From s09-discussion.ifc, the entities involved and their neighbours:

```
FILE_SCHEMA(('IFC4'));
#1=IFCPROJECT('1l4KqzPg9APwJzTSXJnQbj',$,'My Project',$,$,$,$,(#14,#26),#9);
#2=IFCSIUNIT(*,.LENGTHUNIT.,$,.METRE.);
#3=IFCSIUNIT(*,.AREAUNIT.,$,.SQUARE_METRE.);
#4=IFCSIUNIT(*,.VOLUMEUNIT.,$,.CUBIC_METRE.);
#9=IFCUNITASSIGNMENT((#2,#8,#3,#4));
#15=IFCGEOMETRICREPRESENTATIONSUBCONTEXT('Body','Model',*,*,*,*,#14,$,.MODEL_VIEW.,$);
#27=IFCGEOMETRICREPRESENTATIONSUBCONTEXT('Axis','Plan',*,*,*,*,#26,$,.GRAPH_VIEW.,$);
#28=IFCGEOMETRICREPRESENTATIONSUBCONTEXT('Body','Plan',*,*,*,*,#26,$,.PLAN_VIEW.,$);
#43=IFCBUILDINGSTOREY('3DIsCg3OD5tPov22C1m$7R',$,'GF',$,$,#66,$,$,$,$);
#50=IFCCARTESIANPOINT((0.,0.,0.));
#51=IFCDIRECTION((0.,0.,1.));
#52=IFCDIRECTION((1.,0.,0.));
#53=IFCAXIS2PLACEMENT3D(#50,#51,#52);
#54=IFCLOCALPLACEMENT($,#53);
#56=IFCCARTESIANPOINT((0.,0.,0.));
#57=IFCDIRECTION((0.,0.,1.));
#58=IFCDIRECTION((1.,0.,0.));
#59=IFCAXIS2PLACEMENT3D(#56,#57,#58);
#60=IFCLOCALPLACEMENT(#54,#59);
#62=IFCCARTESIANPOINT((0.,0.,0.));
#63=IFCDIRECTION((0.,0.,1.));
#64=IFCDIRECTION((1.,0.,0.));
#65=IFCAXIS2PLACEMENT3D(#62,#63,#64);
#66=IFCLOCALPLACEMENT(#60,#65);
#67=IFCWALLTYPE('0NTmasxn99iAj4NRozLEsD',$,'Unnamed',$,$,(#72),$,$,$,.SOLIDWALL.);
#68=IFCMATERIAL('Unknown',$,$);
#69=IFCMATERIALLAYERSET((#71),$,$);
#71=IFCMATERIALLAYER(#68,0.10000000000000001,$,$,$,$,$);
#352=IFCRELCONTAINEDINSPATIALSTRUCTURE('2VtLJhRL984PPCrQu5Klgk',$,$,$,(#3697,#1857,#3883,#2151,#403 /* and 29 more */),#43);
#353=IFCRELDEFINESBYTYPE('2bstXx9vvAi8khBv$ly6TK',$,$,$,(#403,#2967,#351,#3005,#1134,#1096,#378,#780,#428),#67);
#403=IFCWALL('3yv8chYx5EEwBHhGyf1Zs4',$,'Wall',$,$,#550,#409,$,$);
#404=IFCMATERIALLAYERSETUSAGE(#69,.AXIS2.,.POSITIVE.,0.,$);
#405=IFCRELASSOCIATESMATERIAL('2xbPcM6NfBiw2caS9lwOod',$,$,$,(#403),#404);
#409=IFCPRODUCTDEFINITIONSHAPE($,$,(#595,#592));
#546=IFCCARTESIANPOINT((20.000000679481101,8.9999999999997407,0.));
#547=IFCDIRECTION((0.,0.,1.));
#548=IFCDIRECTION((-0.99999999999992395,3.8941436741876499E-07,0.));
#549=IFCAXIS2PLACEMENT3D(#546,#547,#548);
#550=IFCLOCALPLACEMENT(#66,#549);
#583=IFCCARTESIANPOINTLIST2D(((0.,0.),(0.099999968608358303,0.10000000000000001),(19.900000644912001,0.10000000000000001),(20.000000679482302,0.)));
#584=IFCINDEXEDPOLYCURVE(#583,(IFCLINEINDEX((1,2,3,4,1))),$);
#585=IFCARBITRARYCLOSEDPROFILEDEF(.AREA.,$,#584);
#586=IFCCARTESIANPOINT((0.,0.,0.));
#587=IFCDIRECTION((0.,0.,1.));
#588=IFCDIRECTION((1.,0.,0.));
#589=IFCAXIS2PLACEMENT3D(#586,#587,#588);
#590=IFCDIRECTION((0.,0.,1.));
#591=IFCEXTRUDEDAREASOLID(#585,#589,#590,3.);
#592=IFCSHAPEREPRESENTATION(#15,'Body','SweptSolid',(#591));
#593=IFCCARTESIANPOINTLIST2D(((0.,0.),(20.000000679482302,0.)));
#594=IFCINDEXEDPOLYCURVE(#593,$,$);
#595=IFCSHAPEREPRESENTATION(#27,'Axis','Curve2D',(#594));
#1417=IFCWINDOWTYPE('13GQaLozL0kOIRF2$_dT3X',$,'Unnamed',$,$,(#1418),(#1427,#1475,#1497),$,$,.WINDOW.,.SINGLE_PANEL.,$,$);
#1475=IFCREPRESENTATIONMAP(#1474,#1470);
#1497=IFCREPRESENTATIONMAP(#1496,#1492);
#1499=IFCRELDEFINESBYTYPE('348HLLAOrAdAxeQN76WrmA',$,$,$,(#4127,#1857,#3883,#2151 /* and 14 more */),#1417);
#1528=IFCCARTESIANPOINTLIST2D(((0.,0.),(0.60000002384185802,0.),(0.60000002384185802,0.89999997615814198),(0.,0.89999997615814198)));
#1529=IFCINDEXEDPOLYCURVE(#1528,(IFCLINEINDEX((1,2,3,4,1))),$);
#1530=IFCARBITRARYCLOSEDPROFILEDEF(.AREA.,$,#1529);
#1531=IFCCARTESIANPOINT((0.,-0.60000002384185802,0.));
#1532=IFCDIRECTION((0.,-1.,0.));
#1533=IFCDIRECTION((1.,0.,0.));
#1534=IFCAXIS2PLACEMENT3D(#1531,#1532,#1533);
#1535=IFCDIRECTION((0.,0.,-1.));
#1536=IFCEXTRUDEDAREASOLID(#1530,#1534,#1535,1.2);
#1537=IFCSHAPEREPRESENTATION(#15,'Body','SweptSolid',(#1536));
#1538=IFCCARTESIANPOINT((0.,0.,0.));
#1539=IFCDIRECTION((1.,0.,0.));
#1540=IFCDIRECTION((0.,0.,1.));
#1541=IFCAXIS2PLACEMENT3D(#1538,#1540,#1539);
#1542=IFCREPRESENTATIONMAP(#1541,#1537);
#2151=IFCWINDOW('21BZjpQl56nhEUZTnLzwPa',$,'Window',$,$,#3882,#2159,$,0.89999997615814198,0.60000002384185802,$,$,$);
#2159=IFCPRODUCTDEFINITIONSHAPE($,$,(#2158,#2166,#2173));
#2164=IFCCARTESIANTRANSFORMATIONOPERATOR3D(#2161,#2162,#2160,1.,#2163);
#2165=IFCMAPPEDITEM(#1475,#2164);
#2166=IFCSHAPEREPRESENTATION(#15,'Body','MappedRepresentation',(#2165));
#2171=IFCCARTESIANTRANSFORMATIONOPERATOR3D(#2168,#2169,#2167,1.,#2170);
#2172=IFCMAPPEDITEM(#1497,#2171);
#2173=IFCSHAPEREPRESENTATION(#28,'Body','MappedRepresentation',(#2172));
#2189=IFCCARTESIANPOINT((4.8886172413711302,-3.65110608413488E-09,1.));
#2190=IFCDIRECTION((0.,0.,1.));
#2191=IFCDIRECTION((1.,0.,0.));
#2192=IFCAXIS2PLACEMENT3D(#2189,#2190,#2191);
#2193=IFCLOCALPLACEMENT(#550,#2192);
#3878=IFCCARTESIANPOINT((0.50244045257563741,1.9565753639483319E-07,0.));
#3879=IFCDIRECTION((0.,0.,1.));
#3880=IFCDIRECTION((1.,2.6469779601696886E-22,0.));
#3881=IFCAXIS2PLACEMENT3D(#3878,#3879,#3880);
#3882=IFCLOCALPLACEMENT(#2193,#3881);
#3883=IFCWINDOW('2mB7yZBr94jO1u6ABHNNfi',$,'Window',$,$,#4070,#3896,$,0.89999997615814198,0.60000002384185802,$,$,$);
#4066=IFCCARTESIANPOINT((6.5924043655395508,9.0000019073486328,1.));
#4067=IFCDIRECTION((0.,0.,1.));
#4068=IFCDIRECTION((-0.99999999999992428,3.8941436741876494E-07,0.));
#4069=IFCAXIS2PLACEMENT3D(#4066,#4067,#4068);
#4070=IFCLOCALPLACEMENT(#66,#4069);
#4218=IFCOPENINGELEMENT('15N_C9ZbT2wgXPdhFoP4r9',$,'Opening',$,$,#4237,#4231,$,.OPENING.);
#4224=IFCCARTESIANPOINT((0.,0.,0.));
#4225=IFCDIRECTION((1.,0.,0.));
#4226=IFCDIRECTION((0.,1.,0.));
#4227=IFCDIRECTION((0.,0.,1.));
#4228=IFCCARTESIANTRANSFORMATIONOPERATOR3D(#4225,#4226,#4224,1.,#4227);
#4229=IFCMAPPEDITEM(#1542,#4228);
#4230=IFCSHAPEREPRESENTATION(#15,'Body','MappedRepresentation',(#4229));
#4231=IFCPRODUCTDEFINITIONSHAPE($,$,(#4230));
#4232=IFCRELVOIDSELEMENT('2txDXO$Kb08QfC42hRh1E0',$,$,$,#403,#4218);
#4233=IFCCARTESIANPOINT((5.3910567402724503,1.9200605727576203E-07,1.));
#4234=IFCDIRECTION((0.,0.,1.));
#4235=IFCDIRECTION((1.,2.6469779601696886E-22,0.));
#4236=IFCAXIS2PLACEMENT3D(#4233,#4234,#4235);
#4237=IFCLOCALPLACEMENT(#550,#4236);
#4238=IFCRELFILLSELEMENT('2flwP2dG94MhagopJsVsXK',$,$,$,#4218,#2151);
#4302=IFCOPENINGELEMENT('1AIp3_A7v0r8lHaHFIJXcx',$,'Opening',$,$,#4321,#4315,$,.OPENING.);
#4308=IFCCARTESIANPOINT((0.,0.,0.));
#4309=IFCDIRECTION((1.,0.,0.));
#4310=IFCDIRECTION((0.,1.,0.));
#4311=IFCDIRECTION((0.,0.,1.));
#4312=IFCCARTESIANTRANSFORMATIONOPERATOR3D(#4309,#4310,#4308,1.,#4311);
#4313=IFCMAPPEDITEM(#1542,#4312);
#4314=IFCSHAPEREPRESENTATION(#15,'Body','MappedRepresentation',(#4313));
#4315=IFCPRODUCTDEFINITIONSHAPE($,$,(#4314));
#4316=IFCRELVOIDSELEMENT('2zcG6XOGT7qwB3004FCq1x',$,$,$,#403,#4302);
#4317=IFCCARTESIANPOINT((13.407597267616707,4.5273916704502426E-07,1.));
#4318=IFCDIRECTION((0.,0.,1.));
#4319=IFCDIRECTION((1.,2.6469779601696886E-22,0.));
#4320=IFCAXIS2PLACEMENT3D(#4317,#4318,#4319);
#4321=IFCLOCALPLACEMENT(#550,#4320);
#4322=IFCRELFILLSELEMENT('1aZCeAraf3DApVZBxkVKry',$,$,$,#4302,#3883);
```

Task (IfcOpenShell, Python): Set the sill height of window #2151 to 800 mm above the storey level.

```python
import numpy as np
import ifcopenshell
import ifcopenshell.api.geometry
import ifcopenshell.geom
import ifcopenshell.util.element
import ifcopenshell.util.placement
import ifcopenshell.util.shape
import ifcopenshell.util.unit

model = ifcopenshell.open("s09-discussion.ifc")
unit_scale = ifcopenshell.util.unit.calculate_unit_scale(model)

window = model.by_guid("21BZjpQl56nhEUZTnLzwPa")
opening = window.FillsVoids[0].RelatingOpeningElement
storey = ifcopenshell.util.element.get_container(window, ifc_class="IfcBuildingStorey")
level = ifcopenshell.util.placement.get_local_placement(storey.ObjectPlacement)[2, 3]

# The opening's origin need not be at the sill, so measure its lowest point.
shape = ifcopenshell.geom.create_shape(ifcopenshell.geom.settings(), opening)
bottom = ifcopenshell.util.shape.get_shape_bottom_elevation(shape, shape.geometry) / unit_scale
dz = level + 0.8 - bottom

shift = np.array([0.0, 0.0, dz])
# The window is not placed relative to its opening, so move both.
for product in (opening, window):
    matrix = ifcopenshell.util.placement.get_local_placement(product.ObjectPlacement)
    matrix[:3, 3] += shift
    ifcopenshell.api.geometry.edit_object_placement(model, product=product, matrix=matrix, is_si=False)

print(f"moved by {dz * unit_scale:+.3f} m")

model.write("s09-discussion_v2.ifc")
```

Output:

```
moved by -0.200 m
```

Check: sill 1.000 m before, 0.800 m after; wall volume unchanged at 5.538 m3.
